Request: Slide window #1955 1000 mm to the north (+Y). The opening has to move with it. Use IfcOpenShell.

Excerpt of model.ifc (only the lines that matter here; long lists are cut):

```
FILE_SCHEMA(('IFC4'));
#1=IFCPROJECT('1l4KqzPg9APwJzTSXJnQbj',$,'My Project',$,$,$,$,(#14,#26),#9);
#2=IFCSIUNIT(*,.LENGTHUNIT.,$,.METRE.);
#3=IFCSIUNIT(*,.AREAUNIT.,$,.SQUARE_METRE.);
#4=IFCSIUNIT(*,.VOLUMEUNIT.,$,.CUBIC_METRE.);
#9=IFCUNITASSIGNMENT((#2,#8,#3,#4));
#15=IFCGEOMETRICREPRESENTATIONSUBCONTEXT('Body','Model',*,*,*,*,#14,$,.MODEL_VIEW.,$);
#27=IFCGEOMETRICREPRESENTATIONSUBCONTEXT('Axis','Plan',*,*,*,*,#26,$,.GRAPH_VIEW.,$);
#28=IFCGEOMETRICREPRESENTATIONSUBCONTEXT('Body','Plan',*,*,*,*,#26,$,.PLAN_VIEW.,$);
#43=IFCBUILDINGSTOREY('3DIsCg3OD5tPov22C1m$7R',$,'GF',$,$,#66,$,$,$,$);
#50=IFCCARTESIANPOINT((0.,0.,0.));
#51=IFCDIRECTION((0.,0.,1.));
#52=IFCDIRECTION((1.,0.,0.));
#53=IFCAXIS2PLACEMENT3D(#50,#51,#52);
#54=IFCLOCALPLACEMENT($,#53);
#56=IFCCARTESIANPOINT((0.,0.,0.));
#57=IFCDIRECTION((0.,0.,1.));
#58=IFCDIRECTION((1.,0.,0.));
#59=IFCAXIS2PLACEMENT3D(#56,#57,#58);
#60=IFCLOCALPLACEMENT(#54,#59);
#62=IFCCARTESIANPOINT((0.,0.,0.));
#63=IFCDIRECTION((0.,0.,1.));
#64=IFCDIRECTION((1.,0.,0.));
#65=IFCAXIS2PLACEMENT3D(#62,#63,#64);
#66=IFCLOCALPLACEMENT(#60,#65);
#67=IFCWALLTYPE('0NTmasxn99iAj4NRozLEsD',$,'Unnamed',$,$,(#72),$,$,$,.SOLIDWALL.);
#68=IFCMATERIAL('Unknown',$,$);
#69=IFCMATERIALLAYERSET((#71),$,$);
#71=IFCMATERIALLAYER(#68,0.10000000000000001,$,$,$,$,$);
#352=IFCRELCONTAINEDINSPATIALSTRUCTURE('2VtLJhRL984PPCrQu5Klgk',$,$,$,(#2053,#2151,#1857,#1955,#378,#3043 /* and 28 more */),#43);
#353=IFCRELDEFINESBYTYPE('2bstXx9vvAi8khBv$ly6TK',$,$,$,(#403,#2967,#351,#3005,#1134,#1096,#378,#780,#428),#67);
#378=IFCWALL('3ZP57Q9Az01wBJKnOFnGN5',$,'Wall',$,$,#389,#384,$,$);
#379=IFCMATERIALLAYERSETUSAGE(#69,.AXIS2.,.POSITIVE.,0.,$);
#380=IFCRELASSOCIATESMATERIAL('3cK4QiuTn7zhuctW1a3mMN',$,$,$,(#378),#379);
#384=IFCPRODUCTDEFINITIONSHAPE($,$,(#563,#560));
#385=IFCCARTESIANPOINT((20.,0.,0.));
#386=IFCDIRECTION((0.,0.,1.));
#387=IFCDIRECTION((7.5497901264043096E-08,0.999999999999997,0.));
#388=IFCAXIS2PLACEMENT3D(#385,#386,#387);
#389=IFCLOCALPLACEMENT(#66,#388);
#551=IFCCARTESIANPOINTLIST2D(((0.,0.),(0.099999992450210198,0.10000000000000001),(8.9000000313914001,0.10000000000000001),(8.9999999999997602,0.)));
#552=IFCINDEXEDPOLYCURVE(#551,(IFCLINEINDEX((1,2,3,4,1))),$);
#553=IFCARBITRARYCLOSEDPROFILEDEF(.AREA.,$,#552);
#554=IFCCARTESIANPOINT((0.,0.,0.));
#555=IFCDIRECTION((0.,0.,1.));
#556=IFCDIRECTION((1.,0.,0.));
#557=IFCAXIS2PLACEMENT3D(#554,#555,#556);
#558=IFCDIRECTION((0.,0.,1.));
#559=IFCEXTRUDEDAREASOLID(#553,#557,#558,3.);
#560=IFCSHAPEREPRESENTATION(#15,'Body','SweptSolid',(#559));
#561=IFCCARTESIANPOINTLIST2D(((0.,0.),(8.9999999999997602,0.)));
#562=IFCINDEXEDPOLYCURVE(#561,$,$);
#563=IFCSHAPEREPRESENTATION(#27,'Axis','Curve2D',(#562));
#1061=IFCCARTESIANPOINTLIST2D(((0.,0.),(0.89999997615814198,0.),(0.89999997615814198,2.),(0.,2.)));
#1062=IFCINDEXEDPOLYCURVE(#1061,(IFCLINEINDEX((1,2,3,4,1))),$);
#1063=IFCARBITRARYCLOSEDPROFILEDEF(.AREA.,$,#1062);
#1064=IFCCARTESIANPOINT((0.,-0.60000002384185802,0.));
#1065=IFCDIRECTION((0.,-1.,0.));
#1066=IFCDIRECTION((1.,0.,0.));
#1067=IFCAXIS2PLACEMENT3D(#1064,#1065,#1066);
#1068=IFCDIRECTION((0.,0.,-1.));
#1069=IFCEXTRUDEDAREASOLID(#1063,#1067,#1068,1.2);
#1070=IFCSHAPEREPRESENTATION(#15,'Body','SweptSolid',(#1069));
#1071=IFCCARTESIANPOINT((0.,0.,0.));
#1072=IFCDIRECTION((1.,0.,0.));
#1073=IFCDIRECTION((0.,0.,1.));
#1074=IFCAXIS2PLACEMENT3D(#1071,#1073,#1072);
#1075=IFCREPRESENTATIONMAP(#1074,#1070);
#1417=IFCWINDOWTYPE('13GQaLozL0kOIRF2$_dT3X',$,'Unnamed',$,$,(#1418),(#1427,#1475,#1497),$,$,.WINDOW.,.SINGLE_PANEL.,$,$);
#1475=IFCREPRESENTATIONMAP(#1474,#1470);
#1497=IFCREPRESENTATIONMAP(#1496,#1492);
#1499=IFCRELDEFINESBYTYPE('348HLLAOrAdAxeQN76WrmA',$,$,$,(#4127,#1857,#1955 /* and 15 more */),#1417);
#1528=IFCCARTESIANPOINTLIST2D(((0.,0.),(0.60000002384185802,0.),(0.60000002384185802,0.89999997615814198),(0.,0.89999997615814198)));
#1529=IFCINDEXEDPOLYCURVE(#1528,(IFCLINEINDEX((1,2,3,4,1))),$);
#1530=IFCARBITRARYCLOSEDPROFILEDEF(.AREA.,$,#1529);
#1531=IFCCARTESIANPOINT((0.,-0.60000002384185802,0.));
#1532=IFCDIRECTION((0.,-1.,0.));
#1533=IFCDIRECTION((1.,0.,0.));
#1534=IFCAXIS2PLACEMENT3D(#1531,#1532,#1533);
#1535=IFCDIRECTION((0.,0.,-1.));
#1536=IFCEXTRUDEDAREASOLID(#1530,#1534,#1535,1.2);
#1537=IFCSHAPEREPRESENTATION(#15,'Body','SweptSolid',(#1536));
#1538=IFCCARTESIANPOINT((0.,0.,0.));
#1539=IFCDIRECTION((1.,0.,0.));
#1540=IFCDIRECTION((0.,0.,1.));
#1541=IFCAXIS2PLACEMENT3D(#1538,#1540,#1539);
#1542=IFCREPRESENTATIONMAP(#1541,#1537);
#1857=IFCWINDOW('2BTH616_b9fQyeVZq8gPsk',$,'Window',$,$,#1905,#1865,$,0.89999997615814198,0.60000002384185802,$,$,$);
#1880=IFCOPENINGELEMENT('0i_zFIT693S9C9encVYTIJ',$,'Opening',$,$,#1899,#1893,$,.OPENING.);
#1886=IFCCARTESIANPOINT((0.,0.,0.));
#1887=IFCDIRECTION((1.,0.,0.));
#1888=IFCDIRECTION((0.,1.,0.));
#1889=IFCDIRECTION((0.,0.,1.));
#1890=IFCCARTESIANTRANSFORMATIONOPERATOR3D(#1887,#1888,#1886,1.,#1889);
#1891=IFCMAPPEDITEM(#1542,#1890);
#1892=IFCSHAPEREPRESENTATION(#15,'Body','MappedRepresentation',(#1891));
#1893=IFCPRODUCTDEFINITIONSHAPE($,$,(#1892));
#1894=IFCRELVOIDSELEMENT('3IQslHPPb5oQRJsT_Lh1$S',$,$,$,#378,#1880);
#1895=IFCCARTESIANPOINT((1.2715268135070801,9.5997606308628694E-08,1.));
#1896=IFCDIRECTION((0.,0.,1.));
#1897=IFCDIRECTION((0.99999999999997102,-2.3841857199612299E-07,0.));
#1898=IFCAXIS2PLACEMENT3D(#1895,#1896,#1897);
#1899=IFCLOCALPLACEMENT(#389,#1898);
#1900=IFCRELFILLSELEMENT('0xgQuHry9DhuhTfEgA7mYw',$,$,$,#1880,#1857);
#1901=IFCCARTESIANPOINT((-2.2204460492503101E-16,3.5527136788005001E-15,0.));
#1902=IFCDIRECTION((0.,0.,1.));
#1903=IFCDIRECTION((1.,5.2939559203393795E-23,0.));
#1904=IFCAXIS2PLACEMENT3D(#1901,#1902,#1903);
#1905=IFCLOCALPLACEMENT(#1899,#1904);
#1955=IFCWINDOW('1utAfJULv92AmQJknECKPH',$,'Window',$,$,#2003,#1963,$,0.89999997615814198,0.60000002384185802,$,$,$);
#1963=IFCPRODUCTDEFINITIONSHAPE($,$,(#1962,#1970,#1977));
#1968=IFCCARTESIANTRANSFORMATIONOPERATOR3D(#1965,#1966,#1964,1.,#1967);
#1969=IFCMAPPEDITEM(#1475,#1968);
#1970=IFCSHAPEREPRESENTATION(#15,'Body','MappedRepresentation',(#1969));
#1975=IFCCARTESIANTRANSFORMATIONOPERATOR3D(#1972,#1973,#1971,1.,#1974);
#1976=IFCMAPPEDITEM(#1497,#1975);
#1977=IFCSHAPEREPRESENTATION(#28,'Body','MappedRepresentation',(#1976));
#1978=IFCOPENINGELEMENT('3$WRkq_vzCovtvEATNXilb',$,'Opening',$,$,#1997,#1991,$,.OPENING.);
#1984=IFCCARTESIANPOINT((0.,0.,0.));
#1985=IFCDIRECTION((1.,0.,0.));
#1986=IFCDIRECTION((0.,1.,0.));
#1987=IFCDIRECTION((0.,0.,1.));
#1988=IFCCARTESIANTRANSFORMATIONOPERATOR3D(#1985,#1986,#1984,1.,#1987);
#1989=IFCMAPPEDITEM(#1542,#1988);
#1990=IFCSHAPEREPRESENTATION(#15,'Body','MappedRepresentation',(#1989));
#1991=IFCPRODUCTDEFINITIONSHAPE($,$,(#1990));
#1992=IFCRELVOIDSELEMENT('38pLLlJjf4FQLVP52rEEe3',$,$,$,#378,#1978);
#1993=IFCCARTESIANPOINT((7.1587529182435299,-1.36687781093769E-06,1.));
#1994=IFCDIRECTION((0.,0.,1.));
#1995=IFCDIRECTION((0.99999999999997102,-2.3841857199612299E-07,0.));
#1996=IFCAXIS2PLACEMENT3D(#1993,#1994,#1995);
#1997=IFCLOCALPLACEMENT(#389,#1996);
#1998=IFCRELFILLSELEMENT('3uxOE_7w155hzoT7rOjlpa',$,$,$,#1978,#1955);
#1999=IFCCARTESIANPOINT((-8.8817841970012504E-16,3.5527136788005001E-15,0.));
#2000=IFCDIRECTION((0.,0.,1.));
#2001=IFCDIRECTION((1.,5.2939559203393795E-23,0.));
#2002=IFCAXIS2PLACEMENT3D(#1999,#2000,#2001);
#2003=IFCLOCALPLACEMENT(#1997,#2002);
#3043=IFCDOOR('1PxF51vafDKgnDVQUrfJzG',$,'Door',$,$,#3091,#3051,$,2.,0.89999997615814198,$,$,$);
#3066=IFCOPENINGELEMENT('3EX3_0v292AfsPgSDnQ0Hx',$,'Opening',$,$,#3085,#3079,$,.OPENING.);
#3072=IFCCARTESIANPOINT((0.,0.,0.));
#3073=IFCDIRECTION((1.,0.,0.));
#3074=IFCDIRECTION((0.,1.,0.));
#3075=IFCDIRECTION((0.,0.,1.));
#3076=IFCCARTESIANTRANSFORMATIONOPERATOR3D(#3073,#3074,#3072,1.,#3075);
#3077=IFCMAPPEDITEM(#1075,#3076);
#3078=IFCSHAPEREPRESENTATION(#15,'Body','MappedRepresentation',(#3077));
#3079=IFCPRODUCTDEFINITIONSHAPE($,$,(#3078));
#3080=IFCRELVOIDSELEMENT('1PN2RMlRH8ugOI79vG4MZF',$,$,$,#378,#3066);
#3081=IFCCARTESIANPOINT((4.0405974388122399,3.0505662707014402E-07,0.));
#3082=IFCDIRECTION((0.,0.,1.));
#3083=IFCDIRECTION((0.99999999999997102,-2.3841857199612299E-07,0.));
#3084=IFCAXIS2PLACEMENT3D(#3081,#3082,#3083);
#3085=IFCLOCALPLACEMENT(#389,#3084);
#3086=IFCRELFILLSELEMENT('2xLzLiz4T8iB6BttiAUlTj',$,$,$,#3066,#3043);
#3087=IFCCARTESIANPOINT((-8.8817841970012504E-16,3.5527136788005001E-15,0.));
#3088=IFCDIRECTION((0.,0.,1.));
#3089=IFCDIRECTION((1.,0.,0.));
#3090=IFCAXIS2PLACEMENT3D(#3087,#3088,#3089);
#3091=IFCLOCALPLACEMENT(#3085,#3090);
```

```python
import ifcopenshell
import ifcopenshell.api.geometry
import ifcopenshell.util.placement
import ifcopenshell.util.unit

model = ifcopenshell.open("model.ifc")
unit_scale = ifcopenshell.util.unit.calculate_unit_scale(model)

window = model.by_id(1955)
opening = window.FillsVoids[0].RelatingOpeningElement
wall = opening.VoidsElements[0].RelatingBuildingElement

wall_matrix = ifcopenshell.util.placement.get_local_placement(wall.ObjectPlacement)
shift = wall_matrix[:3, 0] * 1 / unit_scale
before = ifcopenshell.util.placement.get_local_placement(window.ObjectPlacement)[:3, 3].copy()

# The window is placed relative to its opening, so it follows when the opening moves.
matrix = ifcopenshell.util.placement.get_local_placement(opening.ObjectPlacement)
matrix[:3, 3] += shift
ifcopenshell.api.geometry.edit_object_placement(
    model, product=opening, matrix=matrix, is_si=False, should_transform_children=True
)

after = ifcopenshell.util.placement.get_local_placement(window.ObjectPlacement)[:3, 3]
print("window moved by", (after - before).round(3) + 0.0)

model.write("model-out.ifc")
```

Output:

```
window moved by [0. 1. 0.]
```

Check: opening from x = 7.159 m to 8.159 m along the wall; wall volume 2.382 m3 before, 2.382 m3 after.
